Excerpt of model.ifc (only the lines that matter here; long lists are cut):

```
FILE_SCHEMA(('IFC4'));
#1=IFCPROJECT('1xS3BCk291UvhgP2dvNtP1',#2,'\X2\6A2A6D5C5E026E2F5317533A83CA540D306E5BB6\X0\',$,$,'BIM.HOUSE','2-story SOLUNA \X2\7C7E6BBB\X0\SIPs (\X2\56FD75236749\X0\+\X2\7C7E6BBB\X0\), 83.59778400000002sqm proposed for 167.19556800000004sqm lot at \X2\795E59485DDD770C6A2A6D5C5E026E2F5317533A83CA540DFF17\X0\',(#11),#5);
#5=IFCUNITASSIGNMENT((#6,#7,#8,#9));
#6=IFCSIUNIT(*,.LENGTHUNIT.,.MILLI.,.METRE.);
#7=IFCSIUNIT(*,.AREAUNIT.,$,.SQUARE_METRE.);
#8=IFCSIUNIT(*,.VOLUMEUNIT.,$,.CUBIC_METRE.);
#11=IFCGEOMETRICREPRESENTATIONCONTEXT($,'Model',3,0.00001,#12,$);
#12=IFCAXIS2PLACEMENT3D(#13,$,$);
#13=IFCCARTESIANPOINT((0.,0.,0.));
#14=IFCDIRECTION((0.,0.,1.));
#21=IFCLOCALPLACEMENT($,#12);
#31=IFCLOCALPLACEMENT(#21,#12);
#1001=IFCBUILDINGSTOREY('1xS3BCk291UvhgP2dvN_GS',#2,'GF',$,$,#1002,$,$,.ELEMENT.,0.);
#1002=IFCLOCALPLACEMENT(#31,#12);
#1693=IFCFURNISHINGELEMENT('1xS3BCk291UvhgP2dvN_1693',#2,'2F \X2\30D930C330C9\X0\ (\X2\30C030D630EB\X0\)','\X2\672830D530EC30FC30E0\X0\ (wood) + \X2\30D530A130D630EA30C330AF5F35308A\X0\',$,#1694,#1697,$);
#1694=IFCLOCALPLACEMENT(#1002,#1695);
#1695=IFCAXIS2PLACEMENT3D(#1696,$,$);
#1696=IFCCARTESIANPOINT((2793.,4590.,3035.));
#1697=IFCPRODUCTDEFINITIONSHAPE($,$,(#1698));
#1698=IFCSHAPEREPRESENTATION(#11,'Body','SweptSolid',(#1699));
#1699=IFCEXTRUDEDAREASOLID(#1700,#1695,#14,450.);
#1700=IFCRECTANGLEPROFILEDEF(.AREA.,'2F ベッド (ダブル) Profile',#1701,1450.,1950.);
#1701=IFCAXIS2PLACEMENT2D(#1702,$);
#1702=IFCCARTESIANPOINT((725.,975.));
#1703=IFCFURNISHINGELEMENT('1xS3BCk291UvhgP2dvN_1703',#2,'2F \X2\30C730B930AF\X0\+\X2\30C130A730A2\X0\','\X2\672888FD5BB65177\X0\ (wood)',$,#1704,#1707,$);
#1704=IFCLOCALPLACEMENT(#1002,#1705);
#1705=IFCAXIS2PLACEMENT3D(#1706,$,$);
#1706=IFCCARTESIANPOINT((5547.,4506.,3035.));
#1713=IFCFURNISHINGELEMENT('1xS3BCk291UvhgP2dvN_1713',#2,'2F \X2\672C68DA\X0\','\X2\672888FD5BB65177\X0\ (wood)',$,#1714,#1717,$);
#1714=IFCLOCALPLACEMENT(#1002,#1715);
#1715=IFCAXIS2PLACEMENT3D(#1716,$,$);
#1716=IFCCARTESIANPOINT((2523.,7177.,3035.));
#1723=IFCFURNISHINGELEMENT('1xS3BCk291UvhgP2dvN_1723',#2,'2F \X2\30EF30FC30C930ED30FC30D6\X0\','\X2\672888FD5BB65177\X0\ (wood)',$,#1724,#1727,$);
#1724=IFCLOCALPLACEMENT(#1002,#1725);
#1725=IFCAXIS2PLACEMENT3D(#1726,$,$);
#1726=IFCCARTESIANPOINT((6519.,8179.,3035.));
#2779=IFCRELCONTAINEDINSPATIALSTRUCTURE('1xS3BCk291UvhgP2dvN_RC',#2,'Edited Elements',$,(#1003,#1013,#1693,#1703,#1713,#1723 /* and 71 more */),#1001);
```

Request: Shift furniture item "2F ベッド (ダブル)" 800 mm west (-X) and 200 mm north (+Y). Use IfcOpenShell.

```python
import ifcopenshell
import ifcopenshell.api.geometry
import ifcopenshell.util.placement

model = ifcopenshell.open("model.ifc")

item = model.by_id(1693)
matrix = ifcopenshell.util.placement.get_local_placement(item.ObjectPlacement)
matrix[0, 3] -= 800.0
matrix[1, 3] += 200.0
ifcopenshell.api.geometry.edit_object_placement(model, product=item, matrix=matrix, is_si=False)

print(ifcopenshell.util.placement.get_local_placement(item.ObjectPlacement).round(3) + 0.0)

model.write("model_v2.ifc")
```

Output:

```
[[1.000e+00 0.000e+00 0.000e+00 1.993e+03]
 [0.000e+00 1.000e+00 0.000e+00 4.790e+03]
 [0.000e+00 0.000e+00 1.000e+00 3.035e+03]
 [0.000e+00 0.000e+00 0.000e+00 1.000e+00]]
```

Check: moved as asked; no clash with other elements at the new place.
